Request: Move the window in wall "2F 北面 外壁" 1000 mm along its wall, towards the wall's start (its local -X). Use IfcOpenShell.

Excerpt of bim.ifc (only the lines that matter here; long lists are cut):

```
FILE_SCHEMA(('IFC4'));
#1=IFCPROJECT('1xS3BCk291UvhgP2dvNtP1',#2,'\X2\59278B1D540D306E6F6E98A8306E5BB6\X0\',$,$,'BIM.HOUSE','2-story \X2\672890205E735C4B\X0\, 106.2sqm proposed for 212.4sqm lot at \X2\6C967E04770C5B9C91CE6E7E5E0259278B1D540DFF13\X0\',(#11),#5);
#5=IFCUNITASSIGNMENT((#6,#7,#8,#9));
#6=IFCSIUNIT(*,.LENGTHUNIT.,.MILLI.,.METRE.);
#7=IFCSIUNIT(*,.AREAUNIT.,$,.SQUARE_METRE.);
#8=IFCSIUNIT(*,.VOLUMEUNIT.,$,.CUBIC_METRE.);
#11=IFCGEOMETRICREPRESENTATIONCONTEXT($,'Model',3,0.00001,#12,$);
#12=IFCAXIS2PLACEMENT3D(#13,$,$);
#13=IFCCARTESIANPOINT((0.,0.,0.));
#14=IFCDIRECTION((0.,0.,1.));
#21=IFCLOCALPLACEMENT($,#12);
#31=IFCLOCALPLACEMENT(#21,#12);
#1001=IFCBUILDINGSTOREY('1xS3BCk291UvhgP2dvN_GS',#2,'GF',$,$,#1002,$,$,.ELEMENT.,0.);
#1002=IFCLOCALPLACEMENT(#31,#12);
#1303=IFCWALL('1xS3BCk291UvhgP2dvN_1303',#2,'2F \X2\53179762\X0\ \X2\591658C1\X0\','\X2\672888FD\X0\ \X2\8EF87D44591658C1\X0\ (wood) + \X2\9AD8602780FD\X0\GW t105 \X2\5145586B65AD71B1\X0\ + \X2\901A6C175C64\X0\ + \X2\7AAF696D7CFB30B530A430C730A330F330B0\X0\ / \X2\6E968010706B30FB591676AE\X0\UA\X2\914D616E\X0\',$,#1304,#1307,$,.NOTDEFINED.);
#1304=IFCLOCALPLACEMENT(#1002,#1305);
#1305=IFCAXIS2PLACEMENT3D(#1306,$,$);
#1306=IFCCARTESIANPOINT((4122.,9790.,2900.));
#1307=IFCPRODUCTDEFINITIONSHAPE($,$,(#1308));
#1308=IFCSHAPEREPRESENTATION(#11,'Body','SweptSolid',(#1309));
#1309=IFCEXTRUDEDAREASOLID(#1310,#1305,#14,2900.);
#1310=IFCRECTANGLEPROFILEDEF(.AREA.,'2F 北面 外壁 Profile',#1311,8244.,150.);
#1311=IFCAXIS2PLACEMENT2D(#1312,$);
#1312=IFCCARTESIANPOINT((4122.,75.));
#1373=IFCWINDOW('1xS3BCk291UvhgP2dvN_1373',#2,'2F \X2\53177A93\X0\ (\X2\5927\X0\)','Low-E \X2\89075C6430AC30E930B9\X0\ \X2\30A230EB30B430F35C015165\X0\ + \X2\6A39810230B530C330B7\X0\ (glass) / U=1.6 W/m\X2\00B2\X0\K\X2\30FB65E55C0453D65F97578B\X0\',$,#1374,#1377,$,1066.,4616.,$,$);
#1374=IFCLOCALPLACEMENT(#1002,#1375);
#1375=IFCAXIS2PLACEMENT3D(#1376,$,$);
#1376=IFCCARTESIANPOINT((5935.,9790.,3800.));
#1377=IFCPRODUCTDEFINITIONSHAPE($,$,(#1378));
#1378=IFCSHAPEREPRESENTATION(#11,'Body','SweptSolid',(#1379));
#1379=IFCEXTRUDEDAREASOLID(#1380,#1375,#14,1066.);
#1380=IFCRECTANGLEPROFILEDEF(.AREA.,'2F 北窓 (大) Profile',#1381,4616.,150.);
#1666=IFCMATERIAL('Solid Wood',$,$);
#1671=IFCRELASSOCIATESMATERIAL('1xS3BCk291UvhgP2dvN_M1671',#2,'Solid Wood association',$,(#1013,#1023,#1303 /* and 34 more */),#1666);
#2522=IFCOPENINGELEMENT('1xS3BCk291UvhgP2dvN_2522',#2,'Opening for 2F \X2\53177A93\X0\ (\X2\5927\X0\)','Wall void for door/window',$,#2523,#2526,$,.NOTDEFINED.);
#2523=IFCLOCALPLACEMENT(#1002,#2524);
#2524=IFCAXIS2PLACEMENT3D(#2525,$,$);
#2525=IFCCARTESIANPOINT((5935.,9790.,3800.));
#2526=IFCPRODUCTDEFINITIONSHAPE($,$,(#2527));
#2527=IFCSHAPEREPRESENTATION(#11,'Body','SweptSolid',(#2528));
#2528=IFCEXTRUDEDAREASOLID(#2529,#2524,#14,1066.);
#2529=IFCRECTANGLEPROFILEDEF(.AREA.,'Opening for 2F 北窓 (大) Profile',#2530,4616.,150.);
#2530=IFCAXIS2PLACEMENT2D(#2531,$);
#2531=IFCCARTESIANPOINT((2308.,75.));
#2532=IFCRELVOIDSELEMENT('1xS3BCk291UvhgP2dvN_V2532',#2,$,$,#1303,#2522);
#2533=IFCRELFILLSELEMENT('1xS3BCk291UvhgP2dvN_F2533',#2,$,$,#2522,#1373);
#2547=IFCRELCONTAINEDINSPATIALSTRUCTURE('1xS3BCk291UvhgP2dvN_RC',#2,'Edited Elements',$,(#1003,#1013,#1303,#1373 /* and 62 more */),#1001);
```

```python
import ifcopenshell
import ifcopenshell.api.geometry
import ifcopenshell.util.placement
import ifcopenshell.util.unit

model = ifcopenshell.open("bim.ifc")
unit_scale = ifcopenshell.util.unit.calculate_unit_scale(model)

window = model.by_id(1373)
opening = window.FillsVoids[0].RelatingOpeningElement
wall = opening.VoidsElements[0].RelatingBuildingElement

wall_matrix = ifcopenshell.util.placement.get_local_placement(wall.ObjectPlacement)
shift = wall_matrix[:3, 0] * -1 / unit_scale
before = ifcopenshell.util.placement.get_local_placement(window.ObjectPlacement)[:3, 3].copy()

# The window is not placed relative to its opening, so move both.
for product in (opening, window):
    matrix = ifcopenshell.util.placement.get_local_placement(product.ObjectPlacement)
    matrix[:3, 3] += shift
    ifcopenshell.api.geometry.edit_object_placement(model, product=product, matrix=matrix, is_si=False)

after = ifcopenshell.util.placement.get_local_placement(window.ObjectPlacement)[:3, 3]
print("window moved by", (after - before).round(3) + 0.0)

model.write("bim_updated.ifc")
```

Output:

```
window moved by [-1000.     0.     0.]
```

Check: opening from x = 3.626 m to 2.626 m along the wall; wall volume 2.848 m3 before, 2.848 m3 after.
